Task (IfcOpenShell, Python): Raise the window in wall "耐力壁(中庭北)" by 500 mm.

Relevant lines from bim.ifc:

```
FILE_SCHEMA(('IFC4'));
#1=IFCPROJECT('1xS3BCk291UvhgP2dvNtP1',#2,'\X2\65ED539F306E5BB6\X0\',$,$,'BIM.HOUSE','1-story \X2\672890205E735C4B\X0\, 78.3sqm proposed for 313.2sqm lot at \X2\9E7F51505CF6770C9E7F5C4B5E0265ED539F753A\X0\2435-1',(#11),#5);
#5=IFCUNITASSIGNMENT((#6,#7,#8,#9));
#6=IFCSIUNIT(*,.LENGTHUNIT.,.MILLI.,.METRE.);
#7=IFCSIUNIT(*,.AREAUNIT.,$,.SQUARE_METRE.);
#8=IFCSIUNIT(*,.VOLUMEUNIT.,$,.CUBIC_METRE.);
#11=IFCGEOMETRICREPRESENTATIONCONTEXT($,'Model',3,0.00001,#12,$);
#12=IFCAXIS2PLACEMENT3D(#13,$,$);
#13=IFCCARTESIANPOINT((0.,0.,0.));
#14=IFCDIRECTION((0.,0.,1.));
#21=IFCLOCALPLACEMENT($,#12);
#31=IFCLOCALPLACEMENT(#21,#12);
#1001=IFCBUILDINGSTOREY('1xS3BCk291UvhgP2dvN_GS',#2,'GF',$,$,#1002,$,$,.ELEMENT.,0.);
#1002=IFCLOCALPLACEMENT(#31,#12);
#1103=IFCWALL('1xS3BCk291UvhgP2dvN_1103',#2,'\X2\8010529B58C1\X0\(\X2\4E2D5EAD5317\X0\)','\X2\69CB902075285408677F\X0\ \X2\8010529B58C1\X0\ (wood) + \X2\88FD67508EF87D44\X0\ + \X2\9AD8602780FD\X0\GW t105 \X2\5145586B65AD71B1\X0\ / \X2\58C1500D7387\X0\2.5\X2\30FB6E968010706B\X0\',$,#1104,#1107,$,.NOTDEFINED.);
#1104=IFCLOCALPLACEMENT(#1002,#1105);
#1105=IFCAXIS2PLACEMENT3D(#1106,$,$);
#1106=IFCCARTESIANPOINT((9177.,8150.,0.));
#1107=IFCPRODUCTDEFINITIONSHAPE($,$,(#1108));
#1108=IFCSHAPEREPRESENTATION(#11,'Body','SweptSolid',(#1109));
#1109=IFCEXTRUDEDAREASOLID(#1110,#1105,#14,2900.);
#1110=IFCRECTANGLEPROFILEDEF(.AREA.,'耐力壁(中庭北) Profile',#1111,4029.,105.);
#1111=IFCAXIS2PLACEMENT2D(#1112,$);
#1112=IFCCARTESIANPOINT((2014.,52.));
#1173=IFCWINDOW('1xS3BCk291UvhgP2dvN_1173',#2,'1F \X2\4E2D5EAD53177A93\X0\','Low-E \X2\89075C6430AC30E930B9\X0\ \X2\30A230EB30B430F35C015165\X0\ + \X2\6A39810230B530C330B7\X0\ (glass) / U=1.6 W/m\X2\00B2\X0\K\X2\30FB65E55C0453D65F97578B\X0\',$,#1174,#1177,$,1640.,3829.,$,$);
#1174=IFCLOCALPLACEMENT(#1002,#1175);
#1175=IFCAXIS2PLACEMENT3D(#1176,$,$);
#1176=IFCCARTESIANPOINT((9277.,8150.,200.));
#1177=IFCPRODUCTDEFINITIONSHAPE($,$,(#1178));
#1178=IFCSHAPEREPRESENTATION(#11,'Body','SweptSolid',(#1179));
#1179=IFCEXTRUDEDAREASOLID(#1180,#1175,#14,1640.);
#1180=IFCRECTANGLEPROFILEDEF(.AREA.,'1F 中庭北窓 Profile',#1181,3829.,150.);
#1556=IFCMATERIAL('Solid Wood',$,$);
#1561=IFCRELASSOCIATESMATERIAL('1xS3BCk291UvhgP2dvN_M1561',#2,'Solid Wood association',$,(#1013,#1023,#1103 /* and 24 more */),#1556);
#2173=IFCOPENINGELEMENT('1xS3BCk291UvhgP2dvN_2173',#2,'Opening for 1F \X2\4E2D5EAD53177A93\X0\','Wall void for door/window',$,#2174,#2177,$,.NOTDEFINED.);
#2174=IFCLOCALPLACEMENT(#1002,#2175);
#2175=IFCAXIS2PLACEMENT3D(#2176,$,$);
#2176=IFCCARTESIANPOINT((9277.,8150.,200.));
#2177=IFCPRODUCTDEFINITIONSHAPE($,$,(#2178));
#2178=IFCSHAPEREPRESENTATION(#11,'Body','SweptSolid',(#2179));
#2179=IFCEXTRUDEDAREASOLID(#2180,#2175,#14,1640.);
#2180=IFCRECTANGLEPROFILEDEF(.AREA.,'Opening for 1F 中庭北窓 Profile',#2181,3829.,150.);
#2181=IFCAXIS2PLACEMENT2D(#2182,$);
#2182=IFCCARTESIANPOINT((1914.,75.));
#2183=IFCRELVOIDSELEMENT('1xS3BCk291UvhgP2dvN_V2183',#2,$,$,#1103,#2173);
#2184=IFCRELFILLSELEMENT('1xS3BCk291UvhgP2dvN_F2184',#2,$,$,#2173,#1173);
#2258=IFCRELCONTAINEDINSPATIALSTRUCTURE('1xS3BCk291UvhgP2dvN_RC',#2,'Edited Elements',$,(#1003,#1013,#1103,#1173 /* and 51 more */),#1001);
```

```python
import numpy as np
import ifcopenshell
import ifcopenshell.api.geometry
import ifcopenshell.util.placement
import ifcopenshell.util.unit

model = ifcopenshell.open("bim.ifc")
unit_scale = ifcopenshell.util.unit.calculate_unit_scale(model)

window = model.by_guid("1xS3BCk291UvhgP2dvN_1173")
opening = window.FillsVoids[0].RelatingOpeningElement
dz = 0.5 / unit_scale

shift = np.array([0.0, 0.0, dz])
# The window is not placed relative to its opening, so move both.
for product in (opening, window):
    matrix = ifcopenshell.util.placement.get_local_placement(product.ObjectPlacement)
    matrix[:3, 3] += shift
    ifcopenshell.api.geometry.edit_object_placement(model, product=product, matrix=matrix, is_si=False)

print(f"moved by {dz * unit_scale:+.3f} m")

model.write("bim_v2.ifc")
```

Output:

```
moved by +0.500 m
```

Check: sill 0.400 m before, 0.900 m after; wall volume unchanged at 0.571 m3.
